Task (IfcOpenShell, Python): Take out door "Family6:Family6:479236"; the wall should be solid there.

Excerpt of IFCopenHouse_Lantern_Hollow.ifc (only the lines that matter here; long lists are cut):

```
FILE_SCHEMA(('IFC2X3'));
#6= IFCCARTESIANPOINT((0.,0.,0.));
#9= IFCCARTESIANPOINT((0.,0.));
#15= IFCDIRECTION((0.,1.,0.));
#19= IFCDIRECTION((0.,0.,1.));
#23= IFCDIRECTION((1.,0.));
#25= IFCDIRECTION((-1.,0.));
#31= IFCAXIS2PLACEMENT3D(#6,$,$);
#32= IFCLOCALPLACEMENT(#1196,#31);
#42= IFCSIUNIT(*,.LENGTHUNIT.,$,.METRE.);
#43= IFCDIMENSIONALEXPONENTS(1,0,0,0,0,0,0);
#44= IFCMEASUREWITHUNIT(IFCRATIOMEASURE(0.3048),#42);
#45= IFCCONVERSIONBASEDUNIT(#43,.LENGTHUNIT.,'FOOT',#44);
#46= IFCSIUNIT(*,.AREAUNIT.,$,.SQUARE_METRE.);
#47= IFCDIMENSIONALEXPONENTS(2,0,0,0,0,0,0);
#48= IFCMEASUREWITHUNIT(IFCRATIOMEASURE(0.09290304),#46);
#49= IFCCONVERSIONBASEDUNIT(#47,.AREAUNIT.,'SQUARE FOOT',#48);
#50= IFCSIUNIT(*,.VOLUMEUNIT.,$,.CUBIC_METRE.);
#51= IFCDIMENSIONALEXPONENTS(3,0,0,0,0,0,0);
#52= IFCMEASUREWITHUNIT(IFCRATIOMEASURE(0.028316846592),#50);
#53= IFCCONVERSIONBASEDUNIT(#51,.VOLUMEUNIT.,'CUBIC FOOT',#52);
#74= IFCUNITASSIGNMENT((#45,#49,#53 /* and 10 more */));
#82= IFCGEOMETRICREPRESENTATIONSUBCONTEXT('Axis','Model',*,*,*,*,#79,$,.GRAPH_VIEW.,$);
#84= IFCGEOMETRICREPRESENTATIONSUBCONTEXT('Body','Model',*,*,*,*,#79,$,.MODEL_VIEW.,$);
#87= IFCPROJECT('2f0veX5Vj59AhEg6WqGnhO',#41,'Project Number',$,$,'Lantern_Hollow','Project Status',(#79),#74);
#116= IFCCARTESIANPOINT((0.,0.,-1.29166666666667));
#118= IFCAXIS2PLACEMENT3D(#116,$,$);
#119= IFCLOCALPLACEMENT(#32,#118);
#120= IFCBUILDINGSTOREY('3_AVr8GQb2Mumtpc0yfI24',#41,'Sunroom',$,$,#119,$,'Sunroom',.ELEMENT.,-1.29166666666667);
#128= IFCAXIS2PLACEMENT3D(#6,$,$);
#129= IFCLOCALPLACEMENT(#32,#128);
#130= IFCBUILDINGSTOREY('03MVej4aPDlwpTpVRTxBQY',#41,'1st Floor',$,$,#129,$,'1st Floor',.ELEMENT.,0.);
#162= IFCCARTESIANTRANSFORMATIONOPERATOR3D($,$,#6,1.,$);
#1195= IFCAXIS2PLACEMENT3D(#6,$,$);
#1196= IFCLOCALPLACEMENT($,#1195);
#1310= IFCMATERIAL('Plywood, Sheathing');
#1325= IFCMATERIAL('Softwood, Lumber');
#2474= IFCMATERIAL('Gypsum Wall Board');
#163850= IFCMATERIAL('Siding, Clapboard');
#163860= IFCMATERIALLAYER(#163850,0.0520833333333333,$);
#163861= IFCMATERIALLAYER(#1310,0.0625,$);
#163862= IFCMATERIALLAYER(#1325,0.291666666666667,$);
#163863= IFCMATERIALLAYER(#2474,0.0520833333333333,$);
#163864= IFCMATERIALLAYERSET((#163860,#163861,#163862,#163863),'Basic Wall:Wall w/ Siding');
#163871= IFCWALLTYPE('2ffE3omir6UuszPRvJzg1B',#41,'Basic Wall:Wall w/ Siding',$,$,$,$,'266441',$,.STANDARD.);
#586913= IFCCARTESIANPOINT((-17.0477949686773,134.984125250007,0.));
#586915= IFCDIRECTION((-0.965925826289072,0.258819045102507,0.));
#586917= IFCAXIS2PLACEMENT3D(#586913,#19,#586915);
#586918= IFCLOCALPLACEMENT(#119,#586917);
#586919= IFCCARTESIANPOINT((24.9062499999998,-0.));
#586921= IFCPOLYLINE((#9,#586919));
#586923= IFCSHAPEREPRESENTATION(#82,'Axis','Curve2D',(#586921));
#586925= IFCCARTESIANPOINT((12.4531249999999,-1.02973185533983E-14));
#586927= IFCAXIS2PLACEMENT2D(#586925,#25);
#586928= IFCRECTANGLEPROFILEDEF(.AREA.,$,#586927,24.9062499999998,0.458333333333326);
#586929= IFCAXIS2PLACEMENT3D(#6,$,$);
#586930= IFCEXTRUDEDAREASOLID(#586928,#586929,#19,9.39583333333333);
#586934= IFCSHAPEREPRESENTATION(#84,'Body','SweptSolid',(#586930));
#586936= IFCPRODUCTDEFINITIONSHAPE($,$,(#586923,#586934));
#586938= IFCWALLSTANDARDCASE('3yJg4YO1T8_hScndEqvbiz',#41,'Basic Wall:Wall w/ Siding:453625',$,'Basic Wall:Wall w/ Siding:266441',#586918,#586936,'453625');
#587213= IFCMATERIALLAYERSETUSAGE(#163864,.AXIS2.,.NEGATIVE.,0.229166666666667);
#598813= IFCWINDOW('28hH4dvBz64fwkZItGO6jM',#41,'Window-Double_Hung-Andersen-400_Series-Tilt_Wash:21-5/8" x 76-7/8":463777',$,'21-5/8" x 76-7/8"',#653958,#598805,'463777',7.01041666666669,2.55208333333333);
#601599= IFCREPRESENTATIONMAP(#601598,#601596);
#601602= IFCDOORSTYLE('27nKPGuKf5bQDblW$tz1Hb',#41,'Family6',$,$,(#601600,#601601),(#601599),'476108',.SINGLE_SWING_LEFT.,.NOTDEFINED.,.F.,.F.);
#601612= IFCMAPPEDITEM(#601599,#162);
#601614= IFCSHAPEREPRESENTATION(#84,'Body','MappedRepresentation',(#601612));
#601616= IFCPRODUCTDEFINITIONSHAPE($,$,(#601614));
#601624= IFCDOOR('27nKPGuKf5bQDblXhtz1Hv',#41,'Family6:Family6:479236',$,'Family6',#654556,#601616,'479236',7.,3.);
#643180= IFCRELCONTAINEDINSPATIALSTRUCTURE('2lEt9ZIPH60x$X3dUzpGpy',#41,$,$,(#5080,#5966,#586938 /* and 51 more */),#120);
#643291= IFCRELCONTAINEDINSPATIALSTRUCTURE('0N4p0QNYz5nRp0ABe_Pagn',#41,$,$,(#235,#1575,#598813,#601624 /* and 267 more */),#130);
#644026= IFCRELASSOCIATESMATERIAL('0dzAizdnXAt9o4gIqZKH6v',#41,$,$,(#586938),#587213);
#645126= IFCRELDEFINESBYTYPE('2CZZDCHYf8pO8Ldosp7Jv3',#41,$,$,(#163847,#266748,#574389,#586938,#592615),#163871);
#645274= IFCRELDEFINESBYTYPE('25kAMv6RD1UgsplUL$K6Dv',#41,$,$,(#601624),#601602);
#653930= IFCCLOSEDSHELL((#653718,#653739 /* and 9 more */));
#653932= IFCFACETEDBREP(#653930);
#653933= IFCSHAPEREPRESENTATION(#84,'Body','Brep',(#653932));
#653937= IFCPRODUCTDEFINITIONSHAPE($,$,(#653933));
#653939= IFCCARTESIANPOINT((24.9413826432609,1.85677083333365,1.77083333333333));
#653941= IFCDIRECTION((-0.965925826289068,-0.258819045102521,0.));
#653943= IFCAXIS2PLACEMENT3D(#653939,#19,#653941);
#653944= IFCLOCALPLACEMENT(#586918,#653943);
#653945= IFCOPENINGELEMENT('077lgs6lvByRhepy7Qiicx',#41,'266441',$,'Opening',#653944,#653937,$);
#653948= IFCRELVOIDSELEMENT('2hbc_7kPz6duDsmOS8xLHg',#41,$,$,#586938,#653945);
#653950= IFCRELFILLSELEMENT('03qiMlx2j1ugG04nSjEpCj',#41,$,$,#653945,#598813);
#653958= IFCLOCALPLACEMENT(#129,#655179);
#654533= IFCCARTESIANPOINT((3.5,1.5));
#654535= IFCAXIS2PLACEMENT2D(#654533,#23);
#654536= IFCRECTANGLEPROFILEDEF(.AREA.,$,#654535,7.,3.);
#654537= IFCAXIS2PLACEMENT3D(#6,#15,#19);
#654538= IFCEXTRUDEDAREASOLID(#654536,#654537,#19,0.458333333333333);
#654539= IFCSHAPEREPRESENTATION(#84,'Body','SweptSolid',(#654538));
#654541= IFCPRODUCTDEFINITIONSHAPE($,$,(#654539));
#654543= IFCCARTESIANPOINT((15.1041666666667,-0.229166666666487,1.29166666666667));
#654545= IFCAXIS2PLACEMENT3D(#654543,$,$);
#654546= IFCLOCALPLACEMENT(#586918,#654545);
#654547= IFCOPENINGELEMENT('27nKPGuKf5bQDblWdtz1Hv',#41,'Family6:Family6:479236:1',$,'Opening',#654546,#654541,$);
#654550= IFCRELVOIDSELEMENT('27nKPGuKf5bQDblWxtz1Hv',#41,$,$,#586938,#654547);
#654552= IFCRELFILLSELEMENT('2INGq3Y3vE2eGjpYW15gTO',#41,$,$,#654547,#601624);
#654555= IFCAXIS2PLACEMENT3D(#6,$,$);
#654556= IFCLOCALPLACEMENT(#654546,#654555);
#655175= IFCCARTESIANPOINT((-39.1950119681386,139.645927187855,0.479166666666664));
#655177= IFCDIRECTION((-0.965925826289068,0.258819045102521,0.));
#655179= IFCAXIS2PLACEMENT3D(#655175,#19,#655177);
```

```python
import ifcopenshell
import ifcopenshell.api.feature
import ifcopenshell.api.root
import ifcopenshell.geom
import ifcopenshell.util.shape

model = ifcopenshell.open("IFCopenHouse_Lantern_Hollow.ifc")
settings = ifcopenshell.geom.settings()


def volume(element):
    """Net volume in cubic metres, openings subtracted."""
    shape = ifcopenshell.geom.create_shape(settings, element)
    return ifcopenshell.util.shape.get_volume(shape.geometry)


door = model.by_id(601624)
opening = door.FillsVoids[0].RelatingOpeningElement
wall = opening.VoidsElements[0].RelatingBuildingElement
before = volume(wall)

ifcopenshell.api.root.remove_product(model, product=door)
ifcopenshell.api.feature.remove_feature(model, feature=opening)

after = volume(wall)

print(f"wall volume {before:.3f} -> {after:.3f} m3")

model.write("IFCopenHouse_Lantern_Hollow-out.ifc")
```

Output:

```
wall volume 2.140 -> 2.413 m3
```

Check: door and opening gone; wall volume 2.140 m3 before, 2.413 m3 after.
